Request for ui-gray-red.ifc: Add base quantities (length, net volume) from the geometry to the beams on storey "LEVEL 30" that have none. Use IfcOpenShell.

First a look at what the model holds.

```python
import ifcopenshell
import ifcopenshell.util.element
import ifcopenshell.util.unit

model = ifcopenshell.open("ui-gray-red.ifc")
print(model.schema)
for unit_type in ("LENGTHUNIT", "AREAUNIT", "VOLUMEUNIT"):
    print(unit_type, ifcopenshell.util.unit.calculate_unit_scale(model, unit_type))
storey = next(s for s in model.by_type("IfcBuildingStorey") if s.Name == "LEVEL 30")
beams = [e for e in ifcopenshell.util.element.get_decomposition(storey) if e.is_a("IfcBeam")]
for e in sorted(beams, key=lambda e: e.id()):
    print(e.id(), e.is_a(), e.Name, list(ifcopenshell.util.element.get_psets(e, qtos_only=True)), sep=" | ")
```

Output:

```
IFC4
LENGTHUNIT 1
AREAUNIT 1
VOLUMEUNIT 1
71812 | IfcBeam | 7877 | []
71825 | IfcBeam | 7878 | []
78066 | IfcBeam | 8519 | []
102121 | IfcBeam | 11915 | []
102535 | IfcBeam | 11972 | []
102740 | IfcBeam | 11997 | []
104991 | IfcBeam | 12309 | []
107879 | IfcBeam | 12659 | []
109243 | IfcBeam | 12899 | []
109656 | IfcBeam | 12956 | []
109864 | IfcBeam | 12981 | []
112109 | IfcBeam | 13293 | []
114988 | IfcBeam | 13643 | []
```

```python
import ifcopenshell
import ifcopenshell.api.pset
import ifcopenshell.geom
import ifcopenshell.util.element
import ifcopenshell.util.shape
import ifcopenshell.util.unit

model = ifcopenshell.open("ui-gray-red.ifc")
unit_scale = ifcopenshell.util.unit.calculate_unit_scale(model)
volume_scale = ifcopenshell.util.unit.calculate_unit_scale(model, "VOLUMEUNIT")
settings = ifcopenshell.geom.settings()

storey = next(s for s in model.by_type("IfcBuildingStorey") if s.Name == "LEVEL 30")
beams = [e for e in ifcopenshell.util.element.get_decomposition(storey) if e.is_a("IfcBeam")]

for e in sorted(beams, key=lambda e: e.id()):
    if ifcopenshell.util.element.get_psets(e, qtos_only=True, should_inherit=False):
        continue
    # Geometry comes back in metres, in the element's own axes.
    shape = ifcopenshell.geom.create_shape(settings, e)
    values = {
        "Length": ifcopenshell.util.shape.get_max_xyz(shape.geometry) / unit_scale,
        "NetVolume": ifcopenshell.util.shape.get_volume(shape.geometry) / volume_scale,
    }
    qto = ifcopenshell.api.pset.add_qto(model, product=e, name="Qto_BeamBaseQuantities")
    ifcopenshell.api.pset.edit_qto(model, qto=qto, properties=values)
    print(e.id(), {k: round(v, 3) for k, v in values.items()})

model.write("ui-gray-red_edited.ifc")
```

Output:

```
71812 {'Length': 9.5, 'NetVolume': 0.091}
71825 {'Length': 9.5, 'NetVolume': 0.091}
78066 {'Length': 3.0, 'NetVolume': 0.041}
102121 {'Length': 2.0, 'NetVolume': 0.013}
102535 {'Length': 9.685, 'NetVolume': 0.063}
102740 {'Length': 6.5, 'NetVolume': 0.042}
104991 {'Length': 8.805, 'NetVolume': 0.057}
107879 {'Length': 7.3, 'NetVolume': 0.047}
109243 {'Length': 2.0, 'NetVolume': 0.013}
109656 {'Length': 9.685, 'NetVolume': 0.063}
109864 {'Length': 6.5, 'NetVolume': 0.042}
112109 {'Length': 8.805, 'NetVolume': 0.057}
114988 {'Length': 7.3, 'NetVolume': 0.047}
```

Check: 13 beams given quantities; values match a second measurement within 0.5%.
